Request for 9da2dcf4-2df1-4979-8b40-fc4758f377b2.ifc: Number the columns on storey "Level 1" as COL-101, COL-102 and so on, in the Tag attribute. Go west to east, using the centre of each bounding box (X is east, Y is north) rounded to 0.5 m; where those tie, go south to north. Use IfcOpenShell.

First a look at what the model holds.

```python
import ifcopenshell
import ifcopenshell.util.element
import ifcopenshell.util.placement

model = ifcopenshell.open("9da2dcf4-2df1-4979-8b40-fc4758f377b2.ifc")
print(model.schema)
storey = next(s for s in model.by_type("IfcBuildingStorey") if s.Name == "Level 1")
columns = [e for e in ifcopenshell.util.element.get_decomposition(storey) if e.is_a("IfcColumn")]
for e in sorted(columns, key=lambda e: e.id()):
    origin = ifcopenshell.util.placement.get_local_placement(e.ObjectPlacement)[:3, 3]
    print(e.id(), e.Tag, e.Name, origin.round(2) + 0.0, sep=" | ")
```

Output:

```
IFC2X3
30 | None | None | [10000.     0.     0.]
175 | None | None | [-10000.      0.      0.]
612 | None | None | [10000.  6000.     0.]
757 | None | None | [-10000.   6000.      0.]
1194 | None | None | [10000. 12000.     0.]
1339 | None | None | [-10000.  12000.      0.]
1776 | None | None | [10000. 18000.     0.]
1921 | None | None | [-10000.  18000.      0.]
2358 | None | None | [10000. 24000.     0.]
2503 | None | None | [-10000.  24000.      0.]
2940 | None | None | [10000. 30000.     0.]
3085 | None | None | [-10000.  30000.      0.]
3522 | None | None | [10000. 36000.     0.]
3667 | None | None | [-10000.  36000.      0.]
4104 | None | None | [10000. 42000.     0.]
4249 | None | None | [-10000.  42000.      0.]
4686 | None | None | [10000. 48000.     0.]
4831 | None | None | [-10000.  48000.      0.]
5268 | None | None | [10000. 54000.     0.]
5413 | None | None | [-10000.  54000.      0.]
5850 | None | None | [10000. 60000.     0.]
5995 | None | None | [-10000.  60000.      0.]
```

```python
import ifcopenshell
import ifcopenshell.geom
import ifcopenshell.util.element
import ifcopenshell.util.shape

model = ifcopenshell.open("9da2dcf4-2df1-4979-8b40-fc4758f377b2.ifc")
settings = ifcopenshell.geom.settings()
settings.set("use-world-coords", True)


def centre(element):
    shape = ifcopenshell.geom.create_shape(settings, element)
    return ifcopenshell.util.shape.get_bbox_centroid(shape.geometry)


storey = next(s for s in model.by_type("IfcBuildingStorey") if s.Name == "Level 1")
columns = [e for e in ifcopenshell.util.element.get_decomposition(storey) if e.is_a("IfcColumn")]

# Insertion points can sit at a corner or the storey origin, so sort by the geometry (in metres).
centres = {e: centre(e) for e in columns}
columns.sort(key=lambda e: (round(centres[e][0] / 0.5), centres[e][1]))

for i, e in enumerate(columns, start=1):
    number = f"COL-1{i:02d}"
    e.Tag = number
    print(e.id(), number)

model.write("9da2dcf4-2df1-4979-8b40-fc4758f377b2-out.ifc")
```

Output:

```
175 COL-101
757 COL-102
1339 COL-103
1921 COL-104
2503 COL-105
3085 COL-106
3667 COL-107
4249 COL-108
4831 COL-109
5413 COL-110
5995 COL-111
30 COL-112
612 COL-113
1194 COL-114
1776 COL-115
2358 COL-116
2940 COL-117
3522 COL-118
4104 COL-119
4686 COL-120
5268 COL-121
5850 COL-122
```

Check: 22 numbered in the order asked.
